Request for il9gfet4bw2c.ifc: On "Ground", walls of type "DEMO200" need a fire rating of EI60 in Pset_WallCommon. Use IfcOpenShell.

First a look at what the model holds.

```python
import ifcopenshell
import ifcopenshell.util.element

model = ifcopenshell.open("il9gfet4bw2c.ifc")
print(model.schema)
storey = next(s for s in model.by_type("IfcBuildingStorey") if s.Name == "Ground")
walls = [e for e in ifcopenshell.util.element.get_decomposition(storey) if e.is_a("IfcWall")]
seen = {}
for e in walls:
    element_type = ifcopenshell.util.element.get_type(e)
    key = (element_type.Name if element_type != e and element_type else None, ifcopenshell.util.element.get_pset(e, "Pset_WallCommon", "FireRating"))
    seen[key] = seen.get(key, 0) + 1
for (name, value), count in sorted(seen.items(), key=str):
    print(count, "x", name, "|", value)
```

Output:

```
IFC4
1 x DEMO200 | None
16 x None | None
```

```python
import ifcopenshell
import ifcopenshell.api.pset
import ifcopenshell.util.element

model = ifcopenshell.open("il9gfet4bw2c.ifc")

storey = next(s for s in model.by_type("IfcBuildingStorey") if s.Name == "Ground")
walls = [e for e in ifcopenshell.util.element.get_decomposition(storey) if e.is_a("IfcWall")]

count = 0
for e in walls:
    element_type = ifcopenshell.util.element.get_type(e)
    if element_type in (None, e) or element_type.Name != "DEMO200":
        continue
    # add_pset returns the element's existing set when there is one.
    pset = ifcopenshell.api.pset.add_pset(model, product=e, name="Pset_WallCommon")
    ifcopenshell.api.pset.edit_pset(model, pset=pset, properties={"FireRating": "EI60"})
    count += 1

print(count, "walls updated")

model.write("il9gfet4bw2c_v2.ifc")
```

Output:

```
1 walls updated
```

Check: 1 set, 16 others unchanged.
